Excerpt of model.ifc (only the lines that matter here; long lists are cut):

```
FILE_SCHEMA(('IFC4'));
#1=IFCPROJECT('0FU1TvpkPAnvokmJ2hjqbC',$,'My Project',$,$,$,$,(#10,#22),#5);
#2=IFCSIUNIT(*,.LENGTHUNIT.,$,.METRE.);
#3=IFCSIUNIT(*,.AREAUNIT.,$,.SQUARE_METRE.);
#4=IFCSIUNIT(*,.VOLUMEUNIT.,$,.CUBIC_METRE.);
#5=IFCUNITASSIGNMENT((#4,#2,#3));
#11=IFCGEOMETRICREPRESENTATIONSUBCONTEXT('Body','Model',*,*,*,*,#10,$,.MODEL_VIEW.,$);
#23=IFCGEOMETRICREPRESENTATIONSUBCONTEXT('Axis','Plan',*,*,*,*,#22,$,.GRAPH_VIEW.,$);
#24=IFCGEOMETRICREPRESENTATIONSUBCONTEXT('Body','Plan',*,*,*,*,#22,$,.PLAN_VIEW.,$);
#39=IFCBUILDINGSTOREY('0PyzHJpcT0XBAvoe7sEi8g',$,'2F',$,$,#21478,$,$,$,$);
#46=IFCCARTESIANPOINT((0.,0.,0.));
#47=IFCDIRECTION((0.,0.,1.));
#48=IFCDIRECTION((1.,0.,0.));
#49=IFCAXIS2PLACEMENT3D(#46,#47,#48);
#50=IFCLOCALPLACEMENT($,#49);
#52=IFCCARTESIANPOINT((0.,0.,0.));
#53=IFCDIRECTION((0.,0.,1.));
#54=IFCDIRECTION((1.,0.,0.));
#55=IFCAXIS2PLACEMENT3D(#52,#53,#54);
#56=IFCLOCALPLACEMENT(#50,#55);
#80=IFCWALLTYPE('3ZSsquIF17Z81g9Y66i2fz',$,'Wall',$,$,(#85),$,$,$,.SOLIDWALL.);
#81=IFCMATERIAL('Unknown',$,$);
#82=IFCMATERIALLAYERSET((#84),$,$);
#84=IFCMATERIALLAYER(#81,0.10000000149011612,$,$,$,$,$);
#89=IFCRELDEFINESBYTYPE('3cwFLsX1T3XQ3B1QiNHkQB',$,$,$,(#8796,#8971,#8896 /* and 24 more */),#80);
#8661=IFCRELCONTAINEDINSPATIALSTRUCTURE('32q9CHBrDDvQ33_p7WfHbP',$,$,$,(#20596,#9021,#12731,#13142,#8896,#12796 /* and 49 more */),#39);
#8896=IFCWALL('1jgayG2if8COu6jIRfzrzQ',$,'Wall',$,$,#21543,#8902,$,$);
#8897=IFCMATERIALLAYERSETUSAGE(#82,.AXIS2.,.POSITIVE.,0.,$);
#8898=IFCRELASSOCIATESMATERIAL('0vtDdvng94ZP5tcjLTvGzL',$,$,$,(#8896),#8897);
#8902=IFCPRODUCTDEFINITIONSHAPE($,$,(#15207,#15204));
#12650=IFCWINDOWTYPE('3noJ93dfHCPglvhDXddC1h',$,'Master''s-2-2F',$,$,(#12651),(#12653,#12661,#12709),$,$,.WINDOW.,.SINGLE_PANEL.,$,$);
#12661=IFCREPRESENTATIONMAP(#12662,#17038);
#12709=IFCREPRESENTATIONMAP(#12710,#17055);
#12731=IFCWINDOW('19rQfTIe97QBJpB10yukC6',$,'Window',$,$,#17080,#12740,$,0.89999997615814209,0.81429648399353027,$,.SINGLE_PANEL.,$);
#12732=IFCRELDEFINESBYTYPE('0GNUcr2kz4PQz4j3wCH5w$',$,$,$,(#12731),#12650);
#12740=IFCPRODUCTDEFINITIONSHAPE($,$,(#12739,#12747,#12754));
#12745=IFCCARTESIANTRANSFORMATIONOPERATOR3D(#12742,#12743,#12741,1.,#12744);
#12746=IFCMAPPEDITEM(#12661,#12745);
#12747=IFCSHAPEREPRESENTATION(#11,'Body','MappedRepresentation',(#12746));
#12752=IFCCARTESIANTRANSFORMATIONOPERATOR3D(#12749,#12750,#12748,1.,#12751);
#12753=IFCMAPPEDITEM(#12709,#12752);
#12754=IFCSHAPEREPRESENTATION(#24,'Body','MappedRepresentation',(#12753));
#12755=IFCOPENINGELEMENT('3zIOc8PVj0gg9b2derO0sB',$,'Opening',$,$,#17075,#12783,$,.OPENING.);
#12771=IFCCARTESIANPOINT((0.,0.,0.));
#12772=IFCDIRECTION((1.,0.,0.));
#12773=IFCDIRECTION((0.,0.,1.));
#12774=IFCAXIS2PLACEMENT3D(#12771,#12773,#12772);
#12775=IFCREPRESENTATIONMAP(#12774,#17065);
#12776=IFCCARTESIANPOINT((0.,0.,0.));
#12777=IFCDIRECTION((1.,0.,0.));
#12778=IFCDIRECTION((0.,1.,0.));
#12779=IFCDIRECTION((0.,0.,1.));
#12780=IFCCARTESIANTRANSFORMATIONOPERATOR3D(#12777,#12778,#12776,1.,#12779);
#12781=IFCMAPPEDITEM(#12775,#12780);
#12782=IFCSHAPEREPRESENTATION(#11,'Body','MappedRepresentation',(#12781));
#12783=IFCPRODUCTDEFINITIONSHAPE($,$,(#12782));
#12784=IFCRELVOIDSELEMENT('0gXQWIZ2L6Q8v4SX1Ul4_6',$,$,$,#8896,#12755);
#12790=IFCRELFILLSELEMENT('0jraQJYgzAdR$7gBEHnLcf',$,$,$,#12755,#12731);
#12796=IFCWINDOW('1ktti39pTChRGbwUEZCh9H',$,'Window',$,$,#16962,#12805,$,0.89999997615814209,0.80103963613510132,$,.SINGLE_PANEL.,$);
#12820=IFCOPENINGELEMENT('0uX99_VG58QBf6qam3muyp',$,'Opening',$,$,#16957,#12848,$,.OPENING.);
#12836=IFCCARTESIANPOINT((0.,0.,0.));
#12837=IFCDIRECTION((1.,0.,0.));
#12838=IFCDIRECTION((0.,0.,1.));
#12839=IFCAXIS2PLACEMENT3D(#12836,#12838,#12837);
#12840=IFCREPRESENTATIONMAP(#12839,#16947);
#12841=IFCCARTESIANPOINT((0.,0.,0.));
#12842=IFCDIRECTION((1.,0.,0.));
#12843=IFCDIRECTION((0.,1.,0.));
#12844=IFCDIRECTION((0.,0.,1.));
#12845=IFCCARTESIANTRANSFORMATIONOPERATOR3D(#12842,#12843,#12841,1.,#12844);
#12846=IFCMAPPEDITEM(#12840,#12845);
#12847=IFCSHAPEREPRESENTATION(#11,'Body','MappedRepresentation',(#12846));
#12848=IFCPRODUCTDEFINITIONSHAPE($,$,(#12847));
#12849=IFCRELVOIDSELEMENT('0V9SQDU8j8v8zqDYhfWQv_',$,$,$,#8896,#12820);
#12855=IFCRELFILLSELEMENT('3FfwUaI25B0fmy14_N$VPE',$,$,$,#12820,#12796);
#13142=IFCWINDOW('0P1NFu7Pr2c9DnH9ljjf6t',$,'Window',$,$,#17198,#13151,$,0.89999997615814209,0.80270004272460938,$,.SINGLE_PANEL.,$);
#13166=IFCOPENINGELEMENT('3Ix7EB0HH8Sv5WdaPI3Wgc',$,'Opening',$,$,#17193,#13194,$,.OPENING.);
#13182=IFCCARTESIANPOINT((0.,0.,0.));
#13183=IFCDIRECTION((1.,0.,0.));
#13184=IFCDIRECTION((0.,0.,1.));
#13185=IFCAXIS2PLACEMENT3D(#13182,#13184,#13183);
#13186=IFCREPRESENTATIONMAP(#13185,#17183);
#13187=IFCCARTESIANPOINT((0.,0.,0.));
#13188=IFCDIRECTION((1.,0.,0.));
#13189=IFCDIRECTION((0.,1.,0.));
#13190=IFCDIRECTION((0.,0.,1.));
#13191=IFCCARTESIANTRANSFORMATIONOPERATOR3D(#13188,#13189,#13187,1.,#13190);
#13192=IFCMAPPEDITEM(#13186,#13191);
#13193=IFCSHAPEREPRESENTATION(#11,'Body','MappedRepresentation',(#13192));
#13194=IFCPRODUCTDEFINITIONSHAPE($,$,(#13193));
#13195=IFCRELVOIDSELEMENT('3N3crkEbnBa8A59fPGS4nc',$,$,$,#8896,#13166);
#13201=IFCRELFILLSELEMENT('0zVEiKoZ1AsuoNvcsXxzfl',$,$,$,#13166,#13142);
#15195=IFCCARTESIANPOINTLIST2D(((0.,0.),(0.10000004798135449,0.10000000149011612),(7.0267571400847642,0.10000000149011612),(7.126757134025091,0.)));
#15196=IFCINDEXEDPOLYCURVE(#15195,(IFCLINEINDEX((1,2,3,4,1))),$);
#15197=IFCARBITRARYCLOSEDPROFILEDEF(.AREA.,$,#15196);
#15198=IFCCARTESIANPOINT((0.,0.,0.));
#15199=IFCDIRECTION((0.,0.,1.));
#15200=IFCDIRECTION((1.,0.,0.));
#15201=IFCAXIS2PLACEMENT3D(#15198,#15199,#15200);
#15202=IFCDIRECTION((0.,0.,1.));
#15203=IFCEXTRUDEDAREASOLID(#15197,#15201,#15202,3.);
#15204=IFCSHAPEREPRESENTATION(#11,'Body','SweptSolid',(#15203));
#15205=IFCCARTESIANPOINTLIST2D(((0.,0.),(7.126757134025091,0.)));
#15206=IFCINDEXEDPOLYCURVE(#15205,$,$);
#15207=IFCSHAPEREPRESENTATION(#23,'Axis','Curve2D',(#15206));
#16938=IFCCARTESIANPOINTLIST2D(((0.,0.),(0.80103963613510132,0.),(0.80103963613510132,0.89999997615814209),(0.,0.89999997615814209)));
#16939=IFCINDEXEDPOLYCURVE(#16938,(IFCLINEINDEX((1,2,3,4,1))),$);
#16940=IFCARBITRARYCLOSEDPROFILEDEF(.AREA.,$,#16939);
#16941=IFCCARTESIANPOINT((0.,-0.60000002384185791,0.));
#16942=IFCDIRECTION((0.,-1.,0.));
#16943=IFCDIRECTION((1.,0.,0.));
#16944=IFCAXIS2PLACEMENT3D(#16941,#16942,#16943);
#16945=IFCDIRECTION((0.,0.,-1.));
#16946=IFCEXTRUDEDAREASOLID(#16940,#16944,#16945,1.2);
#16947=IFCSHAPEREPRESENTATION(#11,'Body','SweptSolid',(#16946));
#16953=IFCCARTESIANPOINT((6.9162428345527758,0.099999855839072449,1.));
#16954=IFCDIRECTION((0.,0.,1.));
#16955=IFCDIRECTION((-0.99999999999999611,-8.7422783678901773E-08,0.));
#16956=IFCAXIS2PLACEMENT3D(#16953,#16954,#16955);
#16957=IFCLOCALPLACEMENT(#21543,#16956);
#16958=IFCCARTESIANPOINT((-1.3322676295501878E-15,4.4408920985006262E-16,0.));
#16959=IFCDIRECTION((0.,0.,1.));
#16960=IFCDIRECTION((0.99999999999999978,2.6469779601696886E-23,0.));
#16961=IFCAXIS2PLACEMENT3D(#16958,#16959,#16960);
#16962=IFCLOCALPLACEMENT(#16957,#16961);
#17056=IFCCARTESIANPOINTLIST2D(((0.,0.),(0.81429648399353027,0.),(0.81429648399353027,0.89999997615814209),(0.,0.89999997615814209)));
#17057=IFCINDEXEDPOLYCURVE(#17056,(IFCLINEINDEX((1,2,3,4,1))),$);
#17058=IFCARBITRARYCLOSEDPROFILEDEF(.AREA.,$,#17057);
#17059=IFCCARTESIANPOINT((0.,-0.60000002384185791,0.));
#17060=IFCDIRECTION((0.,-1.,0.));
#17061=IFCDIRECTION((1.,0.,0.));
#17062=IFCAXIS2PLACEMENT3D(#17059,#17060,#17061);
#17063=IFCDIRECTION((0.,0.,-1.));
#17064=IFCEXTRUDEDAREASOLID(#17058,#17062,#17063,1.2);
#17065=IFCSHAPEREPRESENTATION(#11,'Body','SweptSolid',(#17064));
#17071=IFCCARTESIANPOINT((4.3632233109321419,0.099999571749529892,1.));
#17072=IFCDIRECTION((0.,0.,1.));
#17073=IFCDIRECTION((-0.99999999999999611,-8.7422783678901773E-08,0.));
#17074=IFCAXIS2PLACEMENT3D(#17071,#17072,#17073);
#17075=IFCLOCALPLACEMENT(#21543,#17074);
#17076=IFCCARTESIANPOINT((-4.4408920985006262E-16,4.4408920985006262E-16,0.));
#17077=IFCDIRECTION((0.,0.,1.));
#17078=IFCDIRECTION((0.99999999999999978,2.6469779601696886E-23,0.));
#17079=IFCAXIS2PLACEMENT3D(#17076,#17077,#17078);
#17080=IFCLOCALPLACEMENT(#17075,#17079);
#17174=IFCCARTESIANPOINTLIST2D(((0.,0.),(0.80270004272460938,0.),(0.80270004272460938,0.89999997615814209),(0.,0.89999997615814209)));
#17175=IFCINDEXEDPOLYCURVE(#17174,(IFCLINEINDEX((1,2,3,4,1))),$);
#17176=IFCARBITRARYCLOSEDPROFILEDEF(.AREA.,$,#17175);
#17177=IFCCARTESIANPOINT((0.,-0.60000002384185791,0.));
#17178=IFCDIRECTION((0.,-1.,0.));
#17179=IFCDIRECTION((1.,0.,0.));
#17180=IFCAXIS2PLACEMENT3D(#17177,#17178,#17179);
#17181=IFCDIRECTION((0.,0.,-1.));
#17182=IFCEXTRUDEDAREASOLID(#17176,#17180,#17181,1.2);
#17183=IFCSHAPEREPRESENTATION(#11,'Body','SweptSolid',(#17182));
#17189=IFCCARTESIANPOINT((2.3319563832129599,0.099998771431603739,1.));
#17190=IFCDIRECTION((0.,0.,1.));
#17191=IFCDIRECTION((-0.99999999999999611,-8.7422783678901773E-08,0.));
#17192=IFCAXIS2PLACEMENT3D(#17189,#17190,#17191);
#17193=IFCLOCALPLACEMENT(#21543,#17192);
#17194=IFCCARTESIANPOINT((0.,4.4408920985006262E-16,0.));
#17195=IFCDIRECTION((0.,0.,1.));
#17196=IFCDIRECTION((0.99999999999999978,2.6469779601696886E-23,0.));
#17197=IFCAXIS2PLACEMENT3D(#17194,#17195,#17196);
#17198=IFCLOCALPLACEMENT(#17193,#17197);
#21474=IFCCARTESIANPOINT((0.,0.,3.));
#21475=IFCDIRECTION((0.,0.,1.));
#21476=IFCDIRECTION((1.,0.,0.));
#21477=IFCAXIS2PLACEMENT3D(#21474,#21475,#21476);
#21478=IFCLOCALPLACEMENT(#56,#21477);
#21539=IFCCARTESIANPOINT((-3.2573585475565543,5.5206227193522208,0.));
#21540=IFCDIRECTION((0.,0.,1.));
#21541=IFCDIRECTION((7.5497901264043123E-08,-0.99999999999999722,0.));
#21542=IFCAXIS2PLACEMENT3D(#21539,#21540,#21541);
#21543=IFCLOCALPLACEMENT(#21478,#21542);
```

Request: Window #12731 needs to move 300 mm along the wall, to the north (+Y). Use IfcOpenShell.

```python
import ifcopenshell
import ifcopenshell.api.geometry
import ifcopenshell.util.placement
import ifcopenshell.util.unit

model = ifcopenshell.open("model.ifc")
unit_scale = ifcopenshell.util.unit.calculate_unit_scale(model)

window = model.by_guid("19rQfTIe97QBJpB10yukC6")
opening = window.FillsVoids[0].RelatingOpeningElement
wall = opening.VoidsElements[0].RelatingBuildingElement

wall_matrix = ifcopenshell.util.placement.get_local_placement(wall.ObjectPlacement)
shift = wall_matrix[:3, 0] * -0.3 / unit_scale
before = ifcopenshell.util.placement.get_local_placement(window.ObjectPlacement)[:3, 3].copy()

# The window is placed relative to its opening, so it follows when the opening moves.
matrix = ifcopenshell.util.placement.get_local_placement(opening.ObjectPlacement)
matrix[:3, 3] += shift
ifcopenshell.api.geometry.edit_object_placement(
    model, product=opening, matrix=matrix, is_si=False, should_transform_children=True
)

after = ifcopenshell.util.placement.get_local_placement(window.ObjectPlacement)[:3, 3]
print("window moved by", (after - before).round(3) + 0.0)

model.write("model_v2.ifc")
```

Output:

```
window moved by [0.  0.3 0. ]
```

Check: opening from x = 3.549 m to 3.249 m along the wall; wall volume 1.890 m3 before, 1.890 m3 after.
